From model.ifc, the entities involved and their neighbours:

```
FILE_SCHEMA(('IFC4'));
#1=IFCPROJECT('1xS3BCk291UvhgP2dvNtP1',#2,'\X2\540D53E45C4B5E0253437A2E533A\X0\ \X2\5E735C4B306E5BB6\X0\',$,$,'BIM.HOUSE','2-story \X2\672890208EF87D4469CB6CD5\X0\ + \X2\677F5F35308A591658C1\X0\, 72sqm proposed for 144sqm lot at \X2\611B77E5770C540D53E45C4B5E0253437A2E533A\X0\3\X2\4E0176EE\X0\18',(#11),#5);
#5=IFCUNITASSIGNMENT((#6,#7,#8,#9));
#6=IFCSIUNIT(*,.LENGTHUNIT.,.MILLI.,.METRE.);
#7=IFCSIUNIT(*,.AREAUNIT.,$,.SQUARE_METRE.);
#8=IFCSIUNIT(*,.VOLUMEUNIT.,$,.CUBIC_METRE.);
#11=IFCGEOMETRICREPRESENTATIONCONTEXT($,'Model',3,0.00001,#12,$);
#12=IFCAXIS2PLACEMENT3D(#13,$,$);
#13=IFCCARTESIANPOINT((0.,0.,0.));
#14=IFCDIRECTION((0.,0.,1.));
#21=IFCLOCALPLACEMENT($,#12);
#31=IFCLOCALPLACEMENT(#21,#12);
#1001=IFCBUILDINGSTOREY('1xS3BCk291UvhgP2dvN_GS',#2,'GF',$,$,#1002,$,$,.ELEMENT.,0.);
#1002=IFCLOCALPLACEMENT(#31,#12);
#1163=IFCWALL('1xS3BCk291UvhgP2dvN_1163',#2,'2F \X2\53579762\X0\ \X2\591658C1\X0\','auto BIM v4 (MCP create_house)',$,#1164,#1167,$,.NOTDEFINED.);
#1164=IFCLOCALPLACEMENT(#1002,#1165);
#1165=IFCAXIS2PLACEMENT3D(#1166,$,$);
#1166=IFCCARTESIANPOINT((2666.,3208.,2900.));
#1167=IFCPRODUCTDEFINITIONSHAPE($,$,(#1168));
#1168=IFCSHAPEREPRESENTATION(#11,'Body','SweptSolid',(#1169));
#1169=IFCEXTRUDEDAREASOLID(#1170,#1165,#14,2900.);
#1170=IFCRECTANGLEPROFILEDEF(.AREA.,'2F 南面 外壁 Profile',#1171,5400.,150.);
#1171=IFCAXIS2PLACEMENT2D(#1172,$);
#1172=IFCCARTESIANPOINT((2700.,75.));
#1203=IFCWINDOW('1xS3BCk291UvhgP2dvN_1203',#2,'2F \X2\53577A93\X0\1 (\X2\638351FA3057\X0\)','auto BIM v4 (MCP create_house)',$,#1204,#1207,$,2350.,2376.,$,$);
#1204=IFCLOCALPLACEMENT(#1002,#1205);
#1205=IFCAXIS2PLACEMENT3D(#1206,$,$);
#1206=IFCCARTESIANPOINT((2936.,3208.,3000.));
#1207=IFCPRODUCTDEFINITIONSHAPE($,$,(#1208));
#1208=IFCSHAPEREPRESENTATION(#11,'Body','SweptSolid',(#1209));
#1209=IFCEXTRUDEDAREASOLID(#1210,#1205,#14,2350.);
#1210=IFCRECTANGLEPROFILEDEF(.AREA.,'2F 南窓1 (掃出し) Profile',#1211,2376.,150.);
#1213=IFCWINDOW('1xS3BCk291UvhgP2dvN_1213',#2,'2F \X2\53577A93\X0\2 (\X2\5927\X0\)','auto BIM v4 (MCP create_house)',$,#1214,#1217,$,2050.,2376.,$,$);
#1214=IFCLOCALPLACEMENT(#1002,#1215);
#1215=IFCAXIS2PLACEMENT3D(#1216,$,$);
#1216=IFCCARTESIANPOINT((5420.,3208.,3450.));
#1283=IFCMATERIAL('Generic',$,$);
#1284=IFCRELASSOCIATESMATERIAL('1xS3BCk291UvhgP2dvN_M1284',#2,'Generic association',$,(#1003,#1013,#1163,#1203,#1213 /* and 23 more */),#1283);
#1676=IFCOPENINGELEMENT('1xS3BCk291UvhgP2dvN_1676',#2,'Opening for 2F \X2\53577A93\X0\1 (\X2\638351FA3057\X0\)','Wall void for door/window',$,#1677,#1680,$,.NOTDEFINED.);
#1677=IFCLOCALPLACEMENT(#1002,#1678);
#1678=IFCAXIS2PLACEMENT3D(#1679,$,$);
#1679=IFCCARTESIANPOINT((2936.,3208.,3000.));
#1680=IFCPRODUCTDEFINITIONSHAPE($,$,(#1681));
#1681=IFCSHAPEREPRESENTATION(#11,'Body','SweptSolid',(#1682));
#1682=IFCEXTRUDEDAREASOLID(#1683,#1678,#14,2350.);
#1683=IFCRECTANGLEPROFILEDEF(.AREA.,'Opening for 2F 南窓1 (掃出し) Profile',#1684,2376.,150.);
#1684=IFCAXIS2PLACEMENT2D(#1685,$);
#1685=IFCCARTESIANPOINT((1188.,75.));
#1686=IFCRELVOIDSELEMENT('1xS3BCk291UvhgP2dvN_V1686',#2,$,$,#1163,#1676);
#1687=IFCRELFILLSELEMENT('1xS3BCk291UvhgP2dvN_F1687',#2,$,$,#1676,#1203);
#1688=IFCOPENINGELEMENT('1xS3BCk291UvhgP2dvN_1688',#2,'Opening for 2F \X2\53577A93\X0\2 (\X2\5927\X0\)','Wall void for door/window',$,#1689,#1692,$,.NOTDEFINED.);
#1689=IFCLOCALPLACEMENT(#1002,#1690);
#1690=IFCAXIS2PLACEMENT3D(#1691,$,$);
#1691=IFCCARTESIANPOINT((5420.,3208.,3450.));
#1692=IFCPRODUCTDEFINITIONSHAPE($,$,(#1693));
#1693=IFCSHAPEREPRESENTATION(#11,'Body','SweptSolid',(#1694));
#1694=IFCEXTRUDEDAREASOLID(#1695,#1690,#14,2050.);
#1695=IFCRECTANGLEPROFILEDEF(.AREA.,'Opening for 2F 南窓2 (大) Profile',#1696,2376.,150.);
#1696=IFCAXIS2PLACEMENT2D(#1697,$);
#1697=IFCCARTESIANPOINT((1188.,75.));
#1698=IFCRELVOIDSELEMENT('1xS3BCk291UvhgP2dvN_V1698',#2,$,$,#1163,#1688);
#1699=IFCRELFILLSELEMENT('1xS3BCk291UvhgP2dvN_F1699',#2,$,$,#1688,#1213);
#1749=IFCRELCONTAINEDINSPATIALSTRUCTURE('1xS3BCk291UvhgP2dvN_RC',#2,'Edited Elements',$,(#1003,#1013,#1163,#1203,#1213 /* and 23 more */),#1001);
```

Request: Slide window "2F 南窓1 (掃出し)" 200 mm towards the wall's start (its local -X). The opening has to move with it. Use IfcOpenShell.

```python
import ifcopenshell
import ifcopenshell.api.geometry
import ifcopenshell.util.placement
import ifcopenshell.util.unit

model = ifcopenshell.open("model.ifc")
unit_scale = ifcopenshell.util.unit.calculate_unit_scale(model)

window = model.by_id(1203)
opening = window.FillsVoids[0].RelatingOpeningElement
wall = opening.VoidsElements[0].RelatingBuildingElement

wall_matrix = ifcopenshell.util.placement.get_local_placement(wall.ObjectPlacement)
shift = wall_matrix[:3, 0] * -0.2 / unit_scale
before = ifcopenshell.util.placement.get_local_placement(window.ObjectPlacement)[:3, 3].copy()

# The window is not placed relative to its opening, so move both.
for product in (opening, window):
    matrix = ifcopenshell.util.placement.get_local_placement(product.ObjectPlacement)
    matrix[:3, 3] += shift
    ifcopenshell.api.geometry.edit_object_placement(model, product=product, matrix=matrix, is_si=False)

after = ifcopenshell.util.placement.get_local_placement(window.ObjectPlacement)[:3, 3]
print("window moved by", (after - before).round(3) + 0.0)

model.write("model-out.ifc")
```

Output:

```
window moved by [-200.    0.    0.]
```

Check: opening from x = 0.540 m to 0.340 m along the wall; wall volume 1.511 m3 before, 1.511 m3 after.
